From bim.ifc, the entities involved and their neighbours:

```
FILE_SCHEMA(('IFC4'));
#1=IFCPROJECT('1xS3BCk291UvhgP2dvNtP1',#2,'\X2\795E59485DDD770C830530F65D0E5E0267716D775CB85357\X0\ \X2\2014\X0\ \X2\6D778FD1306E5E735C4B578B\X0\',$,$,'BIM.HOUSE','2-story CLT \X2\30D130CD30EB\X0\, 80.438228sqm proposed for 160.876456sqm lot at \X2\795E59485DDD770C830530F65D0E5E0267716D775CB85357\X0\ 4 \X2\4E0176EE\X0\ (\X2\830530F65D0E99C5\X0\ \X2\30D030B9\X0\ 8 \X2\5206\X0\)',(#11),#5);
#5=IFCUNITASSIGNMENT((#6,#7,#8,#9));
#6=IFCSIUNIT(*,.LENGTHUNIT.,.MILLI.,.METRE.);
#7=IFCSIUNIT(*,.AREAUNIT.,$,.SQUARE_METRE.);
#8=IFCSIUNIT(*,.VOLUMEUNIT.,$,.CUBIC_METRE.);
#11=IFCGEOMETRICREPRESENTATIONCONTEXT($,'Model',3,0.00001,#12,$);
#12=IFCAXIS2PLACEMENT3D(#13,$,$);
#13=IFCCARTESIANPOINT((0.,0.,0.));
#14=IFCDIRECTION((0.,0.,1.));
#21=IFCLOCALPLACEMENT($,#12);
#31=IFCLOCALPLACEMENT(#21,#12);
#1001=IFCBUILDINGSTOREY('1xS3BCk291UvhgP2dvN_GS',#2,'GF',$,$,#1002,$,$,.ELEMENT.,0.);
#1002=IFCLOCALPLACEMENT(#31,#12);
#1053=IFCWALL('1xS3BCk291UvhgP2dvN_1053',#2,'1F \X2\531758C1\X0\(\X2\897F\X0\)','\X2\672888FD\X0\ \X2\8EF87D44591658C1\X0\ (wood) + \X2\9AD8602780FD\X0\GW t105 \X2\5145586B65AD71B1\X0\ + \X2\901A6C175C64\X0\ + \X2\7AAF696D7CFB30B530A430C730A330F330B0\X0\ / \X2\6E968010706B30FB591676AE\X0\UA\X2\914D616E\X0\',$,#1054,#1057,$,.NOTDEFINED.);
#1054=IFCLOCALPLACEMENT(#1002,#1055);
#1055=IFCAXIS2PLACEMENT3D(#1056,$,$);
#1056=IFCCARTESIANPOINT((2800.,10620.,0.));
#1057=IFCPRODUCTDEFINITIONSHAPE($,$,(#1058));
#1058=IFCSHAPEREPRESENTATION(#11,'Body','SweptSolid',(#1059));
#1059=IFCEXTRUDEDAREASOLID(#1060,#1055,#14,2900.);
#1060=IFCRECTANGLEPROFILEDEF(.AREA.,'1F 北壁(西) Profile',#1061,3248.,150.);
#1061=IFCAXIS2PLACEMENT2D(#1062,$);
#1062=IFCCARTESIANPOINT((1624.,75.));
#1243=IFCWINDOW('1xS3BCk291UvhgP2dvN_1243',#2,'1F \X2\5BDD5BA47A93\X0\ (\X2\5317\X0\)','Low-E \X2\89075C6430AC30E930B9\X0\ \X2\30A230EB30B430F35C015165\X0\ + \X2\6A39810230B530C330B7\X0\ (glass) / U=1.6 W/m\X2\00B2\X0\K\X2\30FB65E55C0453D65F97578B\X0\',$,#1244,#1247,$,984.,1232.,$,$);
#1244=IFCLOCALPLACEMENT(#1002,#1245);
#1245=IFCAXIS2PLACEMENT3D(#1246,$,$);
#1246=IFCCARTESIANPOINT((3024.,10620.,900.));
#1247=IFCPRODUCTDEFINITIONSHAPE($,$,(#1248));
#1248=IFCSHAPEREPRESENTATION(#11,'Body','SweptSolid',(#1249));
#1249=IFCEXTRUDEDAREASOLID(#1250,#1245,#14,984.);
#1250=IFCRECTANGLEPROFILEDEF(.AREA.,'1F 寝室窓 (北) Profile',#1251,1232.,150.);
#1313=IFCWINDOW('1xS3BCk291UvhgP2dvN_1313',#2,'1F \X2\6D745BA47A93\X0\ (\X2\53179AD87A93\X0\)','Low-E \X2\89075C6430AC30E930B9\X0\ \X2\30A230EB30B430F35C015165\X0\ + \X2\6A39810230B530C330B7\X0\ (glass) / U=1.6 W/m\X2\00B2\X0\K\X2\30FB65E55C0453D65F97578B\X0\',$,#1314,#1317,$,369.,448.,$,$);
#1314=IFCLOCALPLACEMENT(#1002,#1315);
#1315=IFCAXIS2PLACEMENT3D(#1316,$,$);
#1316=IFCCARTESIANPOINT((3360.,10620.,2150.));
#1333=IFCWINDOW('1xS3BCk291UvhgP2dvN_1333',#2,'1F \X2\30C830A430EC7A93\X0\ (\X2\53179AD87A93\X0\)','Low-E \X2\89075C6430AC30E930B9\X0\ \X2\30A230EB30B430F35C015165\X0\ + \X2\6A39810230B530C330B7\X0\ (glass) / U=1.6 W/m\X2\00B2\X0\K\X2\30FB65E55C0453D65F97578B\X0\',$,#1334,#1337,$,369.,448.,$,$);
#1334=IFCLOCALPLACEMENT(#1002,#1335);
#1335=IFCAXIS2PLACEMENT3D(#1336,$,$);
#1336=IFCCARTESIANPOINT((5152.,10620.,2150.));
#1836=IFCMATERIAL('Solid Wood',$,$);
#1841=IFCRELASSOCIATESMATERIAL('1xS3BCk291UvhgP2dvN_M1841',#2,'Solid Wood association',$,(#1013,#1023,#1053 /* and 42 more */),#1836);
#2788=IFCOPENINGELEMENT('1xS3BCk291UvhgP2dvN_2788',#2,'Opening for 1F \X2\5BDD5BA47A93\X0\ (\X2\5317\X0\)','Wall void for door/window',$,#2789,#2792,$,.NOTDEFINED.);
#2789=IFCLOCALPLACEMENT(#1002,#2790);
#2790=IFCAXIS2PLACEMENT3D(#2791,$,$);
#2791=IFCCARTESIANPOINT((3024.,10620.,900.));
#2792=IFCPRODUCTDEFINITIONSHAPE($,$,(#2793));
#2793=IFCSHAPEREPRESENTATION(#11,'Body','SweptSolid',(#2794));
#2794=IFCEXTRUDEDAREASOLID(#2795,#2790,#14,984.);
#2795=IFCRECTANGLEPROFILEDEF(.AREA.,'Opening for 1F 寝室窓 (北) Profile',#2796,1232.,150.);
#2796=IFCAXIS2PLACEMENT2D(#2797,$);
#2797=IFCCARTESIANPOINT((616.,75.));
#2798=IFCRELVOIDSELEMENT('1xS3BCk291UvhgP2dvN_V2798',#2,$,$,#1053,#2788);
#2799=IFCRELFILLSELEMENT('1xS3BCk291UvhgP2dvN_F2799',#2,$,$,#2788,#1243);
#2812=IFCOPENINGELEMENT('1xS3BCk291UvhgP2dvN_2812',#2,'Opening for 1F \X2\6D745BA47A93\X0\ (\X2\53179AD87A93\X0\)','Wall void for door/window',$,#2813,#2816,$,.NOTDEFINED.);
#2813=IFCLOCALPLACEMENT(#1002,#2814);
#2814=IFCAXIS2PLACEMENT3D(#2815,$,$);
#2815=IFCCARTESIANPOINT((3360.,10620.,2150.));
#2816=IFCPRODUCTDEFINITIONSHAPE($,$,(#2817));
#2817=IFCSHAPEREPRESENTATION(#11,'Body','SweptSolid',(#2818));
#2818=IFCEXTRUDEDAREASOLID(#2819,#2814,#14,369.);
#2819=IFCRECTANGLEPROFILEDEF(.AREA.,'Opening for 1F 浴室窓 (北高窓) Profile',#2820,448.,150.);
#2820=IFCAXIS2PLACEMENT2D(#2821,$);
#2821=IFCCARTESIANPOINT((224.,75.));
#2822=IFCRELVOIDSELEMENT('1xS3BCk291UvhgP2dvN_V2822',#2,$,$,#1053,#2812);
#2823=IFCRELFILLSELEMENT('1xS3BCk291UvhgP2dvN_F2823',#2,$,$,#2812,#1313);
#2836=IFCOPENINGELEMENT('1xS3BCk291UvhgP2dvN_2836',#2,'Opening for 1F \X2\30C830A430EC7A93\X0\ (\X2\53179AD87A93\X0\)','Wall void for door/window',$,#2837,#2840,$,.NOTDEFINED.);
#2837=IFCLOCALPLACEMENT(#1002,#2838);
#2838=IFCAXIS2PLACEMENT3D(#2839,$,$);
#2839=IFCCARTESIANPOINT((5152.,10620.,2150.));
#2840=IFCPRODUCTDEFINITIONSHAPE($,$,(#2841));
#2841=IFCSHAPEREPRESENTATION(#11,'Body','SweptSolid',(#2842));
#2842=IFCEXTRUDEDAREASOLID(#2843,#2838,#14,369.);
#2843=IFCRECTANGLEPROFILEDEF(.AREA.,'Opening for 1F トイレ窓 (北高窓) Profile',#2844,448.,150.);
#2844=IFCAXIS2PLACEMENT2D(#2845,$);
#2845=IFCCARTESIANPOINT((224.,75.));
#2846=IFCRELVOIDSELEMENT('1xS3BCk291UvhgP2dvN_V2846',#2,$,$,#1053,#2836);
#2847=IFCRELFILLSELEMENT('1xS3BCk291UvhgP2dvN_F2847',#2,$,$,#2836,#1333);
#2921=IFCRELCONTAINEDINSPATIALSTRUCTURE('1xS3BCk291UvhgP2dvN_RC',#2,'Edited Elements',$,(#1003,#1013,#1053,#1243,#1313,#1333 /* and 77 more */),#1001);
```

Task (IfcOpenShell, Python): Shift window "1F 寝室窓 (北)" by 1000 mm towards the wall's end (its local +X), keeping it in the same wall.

```python
import ifcopenshell
import ifcopenshell.api.geometry
import ifcopenshell.util.placement
import ifcopenshell.util.unit

model = ifcopenshell.open("bim.ifc")
unit_scale = ifcopenshell.util.unit.calculate_unit_scale(model)

window = model.by_id(1243)
opening = window.FillsVoids[0].RelatingOpeningElement
wall = opening.VoidsElements[0].RelatingBuildingElement

wall_matrix = ifcopenshell.util.placement.get_local_placement(wall.ObjectPlacement)
shift = wall_matrix[:3, 0] * 1 / unit_scale
before = ifcopenshell.util.placement.get_local_placement(window.ObjectPlacement)[:3, 3].copy()

# The window is not placed relative to its opening, so move both.
for product in (opening, window):
    matrix = ifcopenshell.util.placement.get_local_placement(product.ObjectPlacement)
    matrix[:3, 3] += shift
    ifcopenshell.api.geometry.edit_object_placement(model, product=product, matrix=matrix, is_si=False)

after = ifcopenshell.util.placement.get_local_placement(window.ObjectPlacement)[:3, 3]
print("window moved by", (after - before).round(3) + 0.0)

model.write("bim_rev.ifc")
```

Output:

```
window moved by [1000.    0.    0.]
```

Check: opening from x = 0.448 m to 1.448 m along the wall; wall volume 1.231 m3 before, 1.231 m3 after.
